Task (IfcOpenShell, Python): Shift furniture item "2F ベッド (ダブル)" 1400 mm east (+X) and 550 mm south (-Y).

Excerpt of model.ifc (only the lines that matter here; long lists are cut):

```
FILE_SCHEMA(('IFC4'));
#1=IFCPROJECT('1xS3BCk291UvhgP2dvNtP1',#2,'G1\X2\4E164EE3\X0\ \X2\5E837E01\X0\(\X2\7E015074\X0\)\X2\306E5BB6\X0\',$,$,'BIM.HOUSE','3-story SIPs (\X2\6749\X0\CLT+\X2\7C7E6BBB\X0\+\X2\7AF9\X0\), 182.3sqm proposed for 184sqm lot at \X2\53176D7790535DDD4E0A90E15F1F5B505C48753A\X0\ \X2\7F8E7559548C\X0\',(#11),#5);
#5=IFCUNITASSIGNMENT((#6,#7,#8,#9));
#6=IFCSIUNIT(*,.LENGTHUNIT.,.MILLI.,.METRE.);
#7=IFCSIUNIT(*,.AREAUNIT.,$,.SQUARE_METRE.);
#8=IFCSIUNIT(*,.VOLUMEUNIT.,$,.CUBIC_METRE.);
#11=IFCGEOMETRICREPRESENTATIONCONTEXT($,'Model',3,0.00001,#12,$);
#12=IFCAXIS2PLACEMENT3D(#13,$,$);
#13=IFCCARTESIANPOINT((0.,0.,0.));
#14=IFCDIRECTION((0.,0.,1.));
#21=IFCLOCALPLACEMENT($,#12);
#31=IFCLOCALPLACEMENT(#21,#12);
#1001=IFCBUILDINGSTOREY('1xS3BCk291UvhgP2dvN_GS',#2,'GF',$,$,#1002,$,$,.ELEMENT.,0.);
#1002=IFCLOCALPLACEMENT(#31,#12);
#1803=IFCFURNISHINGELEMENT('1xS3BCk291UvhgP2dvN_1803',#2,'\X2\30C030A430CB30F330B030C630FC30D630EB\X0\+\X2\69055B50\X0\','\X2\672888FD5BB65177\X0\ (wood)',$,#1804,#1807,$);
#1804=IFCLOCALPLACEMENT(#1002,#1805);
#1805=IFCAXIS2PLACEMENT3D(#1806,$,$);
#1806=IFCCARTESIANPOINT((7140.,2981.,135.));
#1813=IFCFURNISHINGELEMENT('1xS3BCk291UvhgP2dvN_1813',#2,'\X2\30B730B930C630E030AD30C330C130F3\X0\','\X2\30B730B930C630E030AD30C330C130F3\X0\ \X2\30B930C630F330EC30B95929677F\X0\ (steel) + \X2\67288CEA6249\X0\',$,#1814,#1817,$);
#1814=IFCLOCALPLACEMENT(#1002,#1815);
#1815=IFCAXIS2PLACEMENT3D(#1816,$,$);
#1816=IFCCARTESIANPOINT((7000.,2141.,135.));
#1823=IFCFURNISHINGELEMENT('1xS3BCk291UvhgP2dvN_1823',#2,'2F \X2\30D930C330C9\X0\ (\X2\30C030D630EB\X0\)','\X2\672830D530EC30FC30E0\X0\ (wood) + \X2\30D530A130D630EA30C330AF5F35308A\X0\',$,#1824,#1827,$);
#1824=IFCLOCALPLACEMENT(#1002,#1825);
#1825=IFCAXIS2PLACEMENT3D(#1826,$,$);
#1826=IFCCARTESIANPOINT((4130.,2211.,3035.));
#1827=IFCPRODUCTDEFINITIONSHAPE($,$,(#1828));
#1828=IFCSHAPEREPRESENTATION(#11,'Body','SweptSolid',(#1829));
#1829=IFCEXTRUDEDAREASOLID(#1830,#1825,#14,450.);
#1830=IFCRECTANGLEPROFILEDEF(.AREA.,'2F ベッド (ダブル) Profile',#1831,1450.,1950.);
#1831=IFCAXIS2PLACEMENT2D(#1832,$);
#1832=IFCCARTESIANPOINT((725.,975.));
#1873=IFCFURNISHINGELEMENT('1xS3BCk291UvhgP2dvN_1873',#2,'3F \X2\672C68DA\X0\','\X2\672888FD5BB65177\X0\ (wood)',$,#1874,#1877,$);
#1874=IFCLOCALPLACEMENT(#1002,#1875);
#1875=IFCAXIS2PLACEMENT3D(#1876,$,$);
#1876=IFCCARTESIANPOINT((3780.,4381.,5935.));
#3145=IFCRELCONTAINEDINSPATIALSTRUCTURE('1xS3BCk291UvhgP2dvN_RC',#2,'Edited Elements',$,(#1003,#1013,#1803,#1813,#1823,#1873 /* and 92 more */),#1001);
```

```python
import ifcopenshell
import ifcopenshell.api.geometry
import ifcopenshell.util.placement

model = ifcopenshell.open("model.ifc")

item = model.by_id(1823)
matrix = ifcopenshell.util.placement.get_local_placement(item.ObjectPlacement)
matrix[0, 3] += 1400.0
matrix[1, 3] -= 550.0
ifcopenshell.api.geometry.edit_object_placement(model, product=item, matrix=matrix, is_si=False)

print(ifcopenshell.util.placement.get_local_placement(item.ObjectPlacement).round(3) + 0.0)

model.write("model_edited.ifc")
```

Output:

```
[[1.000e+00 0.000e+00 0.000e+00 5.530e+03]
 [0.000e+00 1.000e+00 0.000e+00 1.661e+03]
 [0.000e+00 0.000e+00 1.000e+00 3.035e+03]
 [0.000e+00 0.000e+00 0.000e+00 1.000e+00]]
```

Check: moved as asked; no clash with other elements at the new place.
